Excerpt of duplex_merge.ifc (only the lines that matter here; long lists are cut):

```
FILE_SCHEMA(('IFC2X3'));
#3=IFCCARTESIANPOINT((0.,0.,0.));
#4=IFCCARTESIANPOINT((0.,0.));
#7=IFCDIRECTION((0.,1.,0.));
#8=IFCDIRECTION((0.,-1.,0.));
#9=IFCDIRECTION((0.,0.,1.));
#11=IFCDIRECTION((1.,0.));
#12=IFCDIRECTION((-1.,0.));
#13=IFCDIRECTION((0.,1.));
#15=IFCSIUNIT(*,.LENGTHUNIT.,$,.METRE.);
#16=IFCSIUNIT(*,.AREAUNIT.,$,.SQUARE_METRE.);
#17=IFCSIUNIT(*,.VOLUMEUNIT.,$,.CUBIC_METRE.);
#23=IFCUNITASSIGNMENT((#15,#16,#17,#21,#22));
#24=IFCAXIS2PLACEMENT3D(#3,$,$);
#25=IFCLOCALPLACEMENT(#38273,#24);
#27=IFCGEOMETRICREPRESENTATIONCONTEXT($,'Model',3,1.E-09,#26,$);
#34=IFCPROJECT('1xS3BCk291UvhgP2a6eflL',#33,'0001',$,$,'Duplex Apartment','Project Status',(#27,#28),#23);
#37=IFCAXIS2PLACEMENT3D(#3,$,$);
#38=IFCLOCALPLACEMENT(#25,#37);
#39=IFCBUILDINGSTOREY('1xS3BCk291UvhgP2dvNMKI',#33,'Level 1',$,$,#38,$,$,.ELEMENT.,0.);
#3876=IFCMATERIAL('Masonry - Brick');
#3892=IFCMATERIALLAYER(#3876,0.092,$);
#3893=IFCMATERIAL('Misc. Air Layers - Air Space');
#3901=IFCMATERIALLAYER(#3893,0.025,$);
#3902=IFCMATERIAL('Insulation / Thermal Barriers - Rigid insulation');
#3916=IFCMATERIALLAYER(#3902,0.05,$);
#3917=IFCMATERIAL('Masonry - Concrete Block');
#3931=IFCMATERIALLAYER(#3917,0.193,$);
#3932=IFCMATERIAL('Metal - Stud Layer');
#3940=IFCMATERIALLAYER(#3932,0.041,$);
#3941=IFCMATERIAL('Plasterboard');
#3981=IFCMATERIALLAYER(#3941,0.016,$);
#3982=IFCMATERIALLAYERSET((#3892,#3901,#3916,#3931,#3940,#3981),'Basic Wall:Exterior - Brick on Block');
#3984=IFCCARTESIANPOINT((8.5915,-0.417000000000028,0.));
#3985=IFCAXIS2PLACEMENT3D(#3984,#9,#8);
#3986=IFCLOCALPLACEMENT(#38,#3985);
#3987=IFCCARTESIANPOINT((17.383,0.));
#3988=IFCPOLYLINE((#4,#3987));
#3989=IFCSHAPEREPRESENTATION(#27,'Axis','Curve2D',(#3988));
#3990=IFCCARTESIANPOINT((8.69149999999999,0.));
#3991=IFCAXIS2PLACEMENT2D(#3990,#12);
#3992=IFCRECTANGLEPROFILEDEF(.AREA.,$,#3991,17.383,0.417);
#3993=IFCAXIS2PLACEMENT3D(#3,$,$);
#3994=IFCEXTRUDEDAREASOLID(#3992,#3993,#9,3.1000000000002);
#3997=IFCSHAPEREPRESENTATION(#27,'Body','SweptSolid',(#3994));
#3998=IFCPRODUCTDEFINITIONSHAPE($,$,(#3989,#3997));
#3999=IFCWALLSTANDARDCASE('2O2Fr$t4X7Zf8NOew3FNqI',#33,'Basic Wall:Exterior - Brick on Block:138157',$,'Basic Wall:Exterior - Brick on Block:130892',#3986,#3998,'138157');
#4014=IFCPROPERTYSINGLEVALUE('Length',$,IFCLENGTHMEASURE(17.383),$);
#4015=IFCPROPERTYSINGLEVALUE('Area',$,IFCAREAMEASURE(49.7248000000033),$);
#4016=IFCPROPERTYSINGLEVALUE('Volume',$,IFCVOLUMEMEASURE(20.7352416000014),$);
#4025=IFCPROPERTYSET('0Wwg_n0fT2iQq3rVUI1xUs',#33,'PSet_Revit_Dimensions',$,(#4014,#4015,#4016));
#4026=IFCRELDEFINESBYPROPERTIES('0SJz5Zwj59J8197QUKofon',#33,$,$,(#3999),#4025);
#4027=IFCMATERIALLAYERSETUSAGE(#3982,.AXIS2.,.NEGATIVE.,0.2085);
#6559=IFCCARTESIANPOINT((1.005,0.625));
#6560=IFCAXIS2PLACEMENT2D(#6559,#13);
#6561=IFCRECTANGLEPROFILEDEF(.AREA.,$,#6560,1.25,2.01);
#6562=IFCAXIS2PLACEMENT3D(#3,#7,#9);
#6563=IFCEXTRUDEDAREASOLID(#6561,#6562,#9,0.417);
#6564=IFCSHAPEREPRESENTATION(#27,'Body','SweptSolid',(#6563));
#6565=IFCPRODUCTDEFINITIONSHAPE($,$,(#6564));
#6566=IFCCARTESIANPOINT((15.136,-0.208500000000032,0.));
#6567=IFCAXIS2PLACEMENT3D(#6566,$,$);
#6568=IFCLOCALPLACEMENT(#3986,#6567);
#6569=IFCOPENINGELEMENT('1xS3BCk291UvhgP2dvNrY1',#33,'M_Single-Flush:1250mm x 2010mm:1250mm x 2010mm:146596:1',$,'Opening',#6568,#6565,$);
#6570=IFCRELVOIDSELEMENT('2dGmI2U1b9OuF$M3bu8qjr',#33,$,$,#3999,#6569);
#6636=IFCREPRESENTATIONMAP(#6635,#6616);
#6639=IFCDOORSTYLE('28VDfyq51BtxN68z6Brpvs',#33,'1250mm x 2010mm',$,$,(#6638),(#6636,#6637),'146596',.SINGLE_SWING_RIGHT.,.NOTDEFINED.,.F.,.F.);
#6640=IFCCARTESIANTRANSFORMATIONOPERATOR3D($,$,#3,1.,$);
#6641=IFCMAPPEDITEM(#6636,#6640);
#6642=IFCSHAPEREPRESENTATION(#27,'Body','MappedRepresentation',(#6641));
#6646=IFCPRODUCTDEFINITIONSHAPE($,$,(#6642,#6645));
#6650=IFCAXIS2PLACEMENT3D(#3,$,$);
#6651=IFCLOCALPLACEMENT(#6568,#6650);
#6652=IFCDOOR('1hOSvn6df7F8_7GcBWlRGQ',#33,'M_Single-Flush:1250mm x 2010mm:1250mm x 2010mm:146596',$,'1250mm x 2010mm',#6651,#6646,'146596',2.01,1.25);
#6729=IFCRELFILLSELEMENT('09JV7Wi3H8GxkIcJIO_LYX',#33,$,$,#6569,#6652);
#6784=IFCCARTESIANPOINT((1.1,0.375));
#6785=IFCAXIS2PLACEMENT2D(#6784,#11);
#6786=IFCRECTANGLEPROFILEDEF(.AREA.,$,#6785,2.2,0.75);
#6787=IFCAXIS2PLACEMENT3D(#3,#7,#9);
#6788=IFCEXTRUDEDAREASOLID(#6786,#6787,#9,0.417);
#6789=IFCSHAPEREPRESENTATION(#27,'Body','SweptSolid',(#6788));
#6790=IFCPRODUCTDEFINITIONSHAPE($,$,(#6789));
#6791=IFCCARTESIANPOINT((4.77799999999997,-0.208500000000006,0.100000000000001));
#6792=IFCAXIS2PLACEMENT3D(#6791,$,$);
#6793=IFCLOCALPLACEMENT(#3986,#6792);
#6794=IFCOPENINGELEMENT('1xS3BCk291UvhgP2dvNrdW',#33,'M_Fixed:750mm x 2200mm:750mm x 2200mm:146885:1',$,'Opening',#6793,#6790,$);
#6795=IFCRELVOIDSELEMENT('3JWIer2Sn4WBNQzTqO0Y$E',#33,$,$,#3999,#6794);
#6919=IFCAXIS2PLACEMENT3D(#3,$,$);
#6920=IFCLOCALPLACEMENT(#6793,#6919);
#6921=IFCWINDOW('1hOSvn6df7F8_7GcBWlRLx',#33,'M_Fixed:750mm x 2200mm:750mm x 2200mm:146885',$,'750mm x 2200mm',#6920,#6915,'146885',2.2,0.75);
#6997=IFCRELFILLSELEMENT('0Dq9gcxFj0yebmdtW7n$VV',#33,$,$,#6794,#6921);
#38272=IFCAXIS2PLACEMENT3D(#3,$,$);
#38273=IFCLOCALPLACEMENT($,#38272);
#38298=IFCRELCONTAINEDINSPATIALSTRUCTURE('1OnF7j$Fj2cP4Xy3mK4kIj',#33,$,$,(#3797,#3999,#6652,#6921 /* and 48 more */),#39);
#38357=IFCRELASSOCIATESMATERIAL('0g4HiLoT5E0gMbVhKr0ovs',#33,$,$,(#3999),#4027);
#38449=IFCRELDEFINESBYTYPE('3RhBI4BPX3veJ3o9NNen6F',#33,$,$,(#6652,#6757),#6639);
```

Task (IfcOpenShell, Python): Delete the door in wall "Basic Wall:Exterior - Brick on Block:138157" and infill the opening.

```python
import ifcopenshell
import ifcopenshell.api.feature
import ifcopenshell.api.pset
import ifcopenshell.api.root
import ifcopenshell.geom
import ifcopenshell.util.element
import ifcopenshell.util.shape
import ifcopenshell.util.unit

model = ifcopenshell.open("duplex_merge.ifc")
area_scale = ifcopenshell.util.unit.calculate_unit_scale(model, "AREAUNIT")
volume_scale = ifcopenshell.util.unit.calculate_unit_scale(model, "VOLUMEUNIT")
settings = ifcopenshell.geom.settings()


def volume(element):
    """Net volume in cubic metres, openings subtracted."""
    shape = ifcopenshell.geom.create_shape(settings, element)
    return ifcopenshell.util.shape.get_volume(shape.geometry)


door = model.by_guid("1hOSvn6df7F8_7GcBWlRGQ")
opening = door.FillsVoids[0].RelatingOpeningElement
wall = opening.VoidsElements[0].RelatingBuildingElement
before = volume(wall)

ifcopenshell.api.root.remove_product(model, product=door)
ifcopenshell.api.feature.remove_feature(model, feature=opening)

after = volume(wall)
thickness = 0.417  # wall thickness in metres

# Update the wall's stored quantities.
pset = model.by_id(ifcopenshell.util.element.get_pset(wall, "PSet_Revit_Dimensions", should_inherit=False)["id"])
ifcopenshell.api.pset.edit_pset(model, pset=pset, properties={
    "Area": model.create_entity("IfcAreaMeasure", after / thickness / area_scale),
    "Volume": model.create_entity("IfcVolumeMeasure", after / volume_scale),
})

print(f"wall volume {before:.3f} -> {after:.3f} m3")

model.write("duplex_merge_v2.ifc")
```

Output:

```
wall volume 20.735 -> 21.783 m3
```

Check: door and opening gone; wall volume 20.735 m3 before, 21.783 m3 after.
